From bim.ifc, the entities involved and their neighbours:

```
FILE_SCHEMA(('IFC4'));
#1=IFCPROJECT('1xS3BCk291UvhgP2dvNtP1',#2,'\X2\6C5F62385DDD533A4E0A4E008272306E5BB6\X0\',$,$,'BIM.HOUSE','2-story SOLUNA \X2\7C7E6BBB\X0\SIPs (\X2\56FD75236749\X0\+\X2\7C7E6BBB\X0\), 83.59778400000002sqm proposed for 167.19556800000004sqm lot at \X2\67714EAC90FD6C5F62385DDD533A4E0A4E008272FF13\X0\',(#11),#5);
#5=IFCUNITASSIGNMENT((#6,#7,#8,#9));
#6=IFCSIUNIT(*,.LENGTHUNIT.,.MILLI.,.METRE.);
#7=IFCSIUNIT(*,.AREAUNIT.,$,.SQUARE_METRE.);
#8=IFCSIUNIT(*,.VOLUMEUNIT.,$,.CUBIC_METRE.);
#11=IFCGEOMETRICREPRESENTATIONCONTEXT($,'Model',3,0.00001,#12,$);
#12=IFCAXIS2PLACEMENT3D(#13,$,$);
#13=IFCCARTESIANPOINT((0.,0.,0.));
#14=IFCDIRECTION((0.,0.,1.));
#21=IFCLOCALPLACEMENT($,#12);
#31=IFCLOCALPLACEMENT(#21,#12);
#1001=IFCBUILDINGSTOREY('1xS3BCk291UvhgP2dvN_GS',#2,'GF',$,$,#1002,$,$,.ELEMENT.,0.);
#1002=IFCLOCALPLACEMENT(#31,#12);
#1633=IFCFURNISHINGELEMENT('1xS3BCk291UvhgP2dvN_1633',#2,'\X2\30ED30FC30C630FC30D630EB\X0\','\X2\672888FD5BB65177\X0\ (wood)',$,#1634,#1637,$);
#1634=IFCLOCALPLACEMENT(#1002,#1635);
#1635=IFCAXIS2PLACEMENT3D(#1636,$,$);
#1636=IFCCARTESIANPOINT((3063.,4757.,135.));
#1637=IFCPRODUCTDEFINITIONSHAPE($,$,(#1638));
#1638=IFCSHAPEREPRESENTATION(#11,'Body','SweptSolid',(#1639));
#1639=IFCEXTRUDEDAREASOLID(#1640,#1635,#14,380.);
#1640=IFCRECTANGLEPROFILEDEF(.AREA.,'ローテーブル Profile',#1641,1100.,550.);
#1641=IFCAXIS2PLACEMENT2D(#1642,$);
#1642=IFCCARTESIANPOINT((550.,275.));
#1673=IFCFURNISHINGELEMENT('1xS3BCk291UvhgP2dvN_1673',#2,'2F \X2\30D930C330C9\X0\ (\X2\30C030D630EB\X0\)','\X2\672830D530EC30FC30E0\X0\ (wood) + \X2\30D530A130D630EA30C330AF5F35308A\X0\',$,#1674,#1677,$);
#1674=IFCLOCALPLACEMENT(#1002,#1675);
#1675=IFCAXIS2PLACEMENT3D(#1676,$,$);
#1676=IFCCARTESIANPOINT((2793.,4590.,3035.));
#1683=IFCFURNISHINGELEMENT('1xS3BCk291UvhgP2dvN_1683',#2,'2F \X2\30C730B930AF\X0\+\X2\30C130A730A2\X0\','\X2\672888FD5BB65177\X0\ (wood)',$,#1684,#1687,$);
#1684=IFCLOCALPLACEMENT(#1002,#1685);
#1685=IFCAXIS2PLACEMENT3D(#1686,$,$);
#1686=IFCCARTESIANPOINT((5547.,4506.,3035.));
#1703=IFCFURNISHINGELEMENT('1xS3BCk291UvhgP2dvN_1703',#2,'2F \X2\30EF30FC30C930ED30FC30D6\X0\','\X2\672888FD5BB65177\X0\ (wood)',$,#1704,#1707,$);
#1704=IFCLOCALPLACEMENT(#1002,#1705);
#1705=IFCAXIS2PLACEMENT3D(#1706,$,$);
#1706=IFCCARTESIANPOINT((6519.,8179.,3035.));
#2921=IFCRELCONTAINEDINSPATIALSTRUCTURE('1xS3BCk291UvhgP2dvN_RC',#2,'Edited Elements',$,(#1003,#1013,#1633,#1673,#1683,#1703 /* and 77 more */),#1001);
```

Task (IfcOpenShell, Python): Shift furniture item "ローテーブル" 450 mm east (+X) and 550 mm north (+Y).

```python
import ifcopenshell
import ifcopenshell.api.geometry
import ifcopenshell.util.placement
import ifcopenshell.util.unit

model = ifcopenshell.open("bim.ifc")
unit_scale = ifcopenshell.util.unit.calculate_unit_scale(model)

item = model.by_guid("1xS3BCk291UvhgP2dvN_1633")
matrix = ifcopenshell.util.placement.get_local_placement(item.ObjectPlacement)
matrix[0, 3] += 0.45 / unit_scale
matrix[1, 3] += 0.55 / unit_scale
ifcopenshell.api.geometry.edit_object_placement(model, product=item, matrix=matrix, is_si=False)

print(ifcopenshell.util.placement.get_local_placement(item.ObjectPlacement).round(3) + 0.0)

model.write("bim_v2.ifc")
```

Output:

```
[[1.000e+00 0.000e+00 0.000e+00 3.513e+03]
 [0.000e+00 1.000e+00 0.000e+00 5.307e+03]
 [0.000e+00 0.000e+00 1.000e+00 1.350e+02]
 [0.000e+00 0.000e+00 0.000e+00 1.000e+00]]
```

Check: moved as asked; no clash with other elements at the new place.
